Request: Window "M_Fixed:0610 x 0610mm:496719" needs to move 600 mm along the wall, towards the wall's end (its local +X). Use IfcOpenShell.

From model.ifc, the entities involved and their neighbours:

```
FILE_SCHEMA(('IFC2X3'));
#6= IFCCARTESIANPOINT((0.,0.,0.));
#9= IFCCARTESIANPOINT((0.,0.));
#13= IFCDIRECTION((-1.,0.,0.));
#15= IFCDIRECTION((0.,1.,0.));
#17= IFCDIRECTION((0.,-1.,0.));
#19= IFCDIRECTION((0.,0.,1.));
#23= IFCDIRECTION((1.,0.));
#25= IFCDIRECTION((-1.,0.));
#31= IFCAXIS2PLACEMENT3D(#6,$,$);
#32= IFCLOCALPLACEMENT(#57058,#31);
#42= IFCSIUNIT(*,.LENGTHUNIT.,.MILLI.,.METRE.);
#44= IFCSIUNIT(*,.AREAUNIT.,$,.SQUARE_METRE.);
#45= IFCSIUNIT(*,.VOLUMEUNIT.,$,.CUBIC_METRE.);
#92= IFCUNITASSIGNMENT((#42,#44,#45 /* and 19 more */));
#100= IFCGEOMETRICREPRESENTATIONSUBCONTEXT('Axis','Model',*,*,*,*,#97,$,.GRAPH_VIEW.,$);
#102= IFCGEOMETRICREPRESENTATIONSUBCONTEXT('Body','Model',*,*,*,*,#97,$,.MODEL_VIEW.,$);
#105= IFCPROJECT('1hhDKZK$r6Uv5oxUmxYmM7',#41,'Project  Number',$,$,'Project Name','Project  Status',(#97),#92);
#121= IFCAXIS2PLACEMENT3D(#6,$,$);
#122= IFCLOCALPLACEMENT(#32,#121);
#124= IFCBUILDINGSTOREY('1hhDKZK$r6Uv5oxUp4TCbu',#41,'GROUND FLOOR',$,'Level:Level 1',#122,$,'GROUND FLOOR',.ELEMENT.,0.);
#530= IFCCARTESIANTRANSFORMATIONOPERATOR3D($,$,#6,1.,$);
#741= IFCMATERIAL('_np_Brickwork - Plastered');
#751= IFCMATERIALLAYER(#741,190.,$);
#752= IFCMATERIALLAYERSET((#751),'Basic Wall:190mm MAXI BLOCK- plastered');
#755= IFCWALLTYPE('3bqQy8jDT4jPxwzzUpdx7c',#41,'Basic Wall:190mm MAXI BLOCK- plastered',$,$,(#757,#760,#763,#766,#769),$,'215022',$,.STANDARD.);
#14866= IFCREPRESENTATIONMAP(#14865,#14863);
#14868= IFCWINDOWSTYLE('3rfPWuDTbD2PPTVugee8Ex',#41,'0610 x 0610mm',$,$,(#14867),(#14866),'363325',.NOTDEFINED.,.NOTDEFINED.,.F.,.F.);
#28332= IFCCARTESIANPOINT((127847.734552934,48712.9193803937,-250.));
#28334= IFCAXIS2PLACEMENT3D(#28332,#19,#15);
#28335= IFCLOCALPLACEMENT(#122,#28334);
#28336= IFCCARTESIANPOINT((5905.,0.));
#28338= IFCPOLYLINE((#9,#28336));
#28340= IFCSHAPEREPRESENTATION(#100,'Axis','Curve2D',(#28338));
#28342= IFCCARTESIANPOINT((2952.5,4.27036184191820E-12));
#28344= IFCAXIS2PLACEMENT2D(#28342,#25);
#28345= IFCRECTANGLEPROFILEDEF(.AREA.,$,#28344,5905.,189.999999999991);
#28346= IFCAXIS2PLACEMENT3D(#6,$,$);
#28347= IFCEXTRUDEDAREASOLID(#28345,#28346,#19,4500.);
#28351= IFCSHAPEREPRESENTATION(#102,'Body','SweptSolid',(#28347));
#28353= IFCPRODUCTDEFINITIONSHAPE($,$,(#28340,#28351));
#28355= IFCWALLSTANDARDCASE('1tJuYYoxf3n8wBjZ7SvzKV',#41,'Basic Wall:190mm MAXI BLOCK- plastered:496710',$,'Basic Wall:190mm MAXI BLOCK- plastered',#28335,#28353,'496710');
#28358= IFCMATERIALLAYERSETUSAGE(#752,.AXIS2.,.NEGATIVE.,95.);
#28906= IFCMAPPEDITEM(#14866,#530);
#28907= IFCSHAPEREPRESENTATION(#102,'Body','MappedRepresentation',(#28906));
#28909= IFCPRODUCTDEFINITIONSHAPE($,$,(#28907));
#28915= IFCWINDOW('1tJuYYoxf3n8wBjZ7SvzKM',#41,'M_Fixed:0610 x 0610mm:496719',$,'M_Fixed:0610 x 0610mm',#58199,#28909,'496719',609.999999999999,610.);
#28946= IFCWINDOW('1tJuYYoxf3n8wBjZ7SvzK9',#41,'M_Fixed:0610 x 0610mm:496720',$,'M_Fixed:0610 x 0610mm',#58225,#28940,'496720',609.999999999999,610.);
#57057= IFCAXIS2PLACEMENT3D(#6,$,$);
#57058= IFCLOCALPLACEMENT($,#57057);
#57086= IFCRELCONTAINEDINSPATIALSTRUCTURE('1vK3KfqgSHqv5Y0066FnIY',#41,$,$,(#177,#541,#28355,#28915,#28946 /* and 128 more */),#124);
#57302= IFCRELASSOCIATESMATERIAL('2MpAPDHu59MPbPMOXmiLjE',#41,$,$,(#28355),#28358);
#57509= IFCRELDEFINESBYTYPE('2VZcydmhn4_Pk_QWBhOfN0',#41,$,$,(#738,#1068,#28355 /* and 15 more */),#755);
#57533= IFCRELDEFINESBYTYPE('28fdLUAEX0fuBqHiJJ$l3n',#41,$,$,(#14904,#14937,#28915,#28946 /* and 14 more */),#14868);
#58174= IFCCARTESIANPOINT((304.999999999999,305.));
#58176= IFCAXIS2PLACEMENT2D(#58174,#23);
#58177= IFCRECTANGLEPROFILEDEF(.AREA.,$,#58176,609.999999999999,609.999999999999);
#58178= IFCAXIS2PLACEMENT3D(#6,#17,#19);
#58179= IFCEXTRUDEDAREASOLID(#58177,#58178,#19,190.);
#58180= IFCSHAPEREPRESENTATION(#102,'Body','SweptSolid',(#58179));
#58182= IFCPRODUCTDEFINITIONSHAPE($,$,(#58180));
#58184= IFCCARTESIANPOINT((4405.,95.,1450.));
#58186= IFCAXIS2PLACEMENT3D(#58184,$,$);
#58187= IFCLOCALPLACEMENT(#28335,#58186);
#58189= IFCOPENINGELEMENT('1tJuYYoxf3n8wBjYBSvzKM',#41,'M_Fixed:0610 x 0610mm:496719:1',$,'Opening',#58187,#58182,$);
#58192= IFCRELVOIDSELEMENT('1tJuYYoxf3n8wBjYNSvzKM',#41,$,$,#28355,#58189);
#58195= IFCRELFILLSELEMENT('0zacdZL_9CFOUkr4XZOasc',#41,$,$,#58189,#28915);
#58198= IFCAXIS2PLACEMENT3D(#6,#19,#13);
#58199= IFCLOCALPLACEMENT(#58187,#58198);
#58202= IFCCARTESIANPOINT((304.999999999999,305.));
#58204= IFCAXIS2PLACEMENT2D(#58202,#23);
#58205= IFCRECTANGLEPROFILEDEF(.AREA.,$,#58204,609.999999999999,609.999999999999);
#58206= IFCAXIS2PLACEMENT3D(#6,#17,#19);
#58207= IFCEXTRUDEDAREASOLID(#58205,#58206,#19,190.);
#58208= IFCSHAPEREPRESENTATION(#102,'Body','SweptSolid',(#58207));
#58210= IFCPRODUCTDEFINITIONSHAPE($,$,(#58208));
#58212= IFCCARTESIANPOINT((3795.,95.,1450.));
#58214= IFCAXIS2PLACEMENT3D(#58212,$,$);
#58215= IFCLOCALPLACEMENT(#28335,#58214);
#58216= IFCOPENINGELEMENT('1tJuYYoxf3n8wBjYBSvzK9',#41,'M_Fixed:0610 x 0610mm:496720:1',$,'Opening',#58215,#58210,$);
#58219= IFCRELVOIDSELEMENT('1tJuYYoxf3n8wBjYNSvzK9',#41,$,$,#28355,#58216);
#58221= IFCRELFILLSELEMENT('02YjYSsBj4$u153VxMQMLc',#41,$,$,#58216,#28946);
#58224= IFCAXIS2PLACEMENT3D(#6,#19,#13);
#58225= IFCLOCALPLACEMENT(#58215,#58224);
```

```python
import ifcopenshell
import ifcopenshell.api.geometry
import ifcopenshell.util.placement

model = ifcopenshell.open("model.ifc")

window = model.by_guid("1tJuYYoxf3n8wBjZ7SvzKM")
opening = window.FillsVoids[0].RelatingOpeningElement
wall = opening.VoidsElements[0].RelatingBuildingElement

wall_matrix = ifcopenshell.util.placement.get_local_placement(wall.ObjectPlacement)
shift = wall_matrix[:3, 0] * 600.0
before = ifcopenshell.util.placement.get_local_placement(window.ObjectPlacement)[:3, 3].copy()

# The window is placed relative to its opening, so it follows when the opening moves.
matrix = ifcopenshell.util.placement.get_local_placement(opening.ObjectPlacement)
matrix[:3, 3] += shift
ifcopenshell.api.geometry.edit_object_placement(
    model, product=opening, matrix=matrix, is_si=False, should_transform_children=True
)

after = ifcopenshell.util.placement.get_local_placement(window.ObjectPlacement)[:3, 3]
print("window moved by", (after - before).round(3) + 0.0)

model.write("model_edited.ifc")
```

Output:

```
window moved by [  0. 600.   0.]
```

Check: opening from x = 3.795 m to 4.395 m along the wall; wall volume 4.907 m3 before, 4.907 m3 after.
